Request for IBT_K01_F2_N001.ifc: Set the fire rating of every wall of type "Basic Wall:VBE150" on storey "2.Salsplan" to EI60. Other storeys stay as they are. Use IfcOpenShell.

First a look at what the model holds.

```python
import ifcopenshell
import ifcopenshell.util.element

model = ifcopenshell.open("IBT_K01_F2_N001.ifc")
print(model.schema)
storey = next(s for s in model.by_type("IfcBuildingStorey") if s.Name == "2.Salsplan")
walls = [e for e in ifcopenshell.util.element.get_decomposition(storey) if e.is_a("IfcWall")]
seen = {}
for e in walls:
    element_type = ifcopenshell.util.element.get_type(e)
    key = (element_type.Name if element_type != e and element_type else None, ifcopenshell.util.element.get_pset(e, "Pset_WallCommon", "FireRating"))
    seen[key] = seen.get(key, 0) + 1
for (name, value), count in sorted(seen.items(), key=str):
    print(count, "x", name, "|", value)
```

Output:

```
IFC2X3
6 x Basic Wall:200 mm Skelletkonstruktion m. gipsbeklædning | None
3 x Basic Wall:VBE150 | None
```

```python
import ifcopenshell
import ifcopenshell.api.pset
import ifcopenshell.util.element

model = ifcopenshell.open("IBT_K01_F2_N001.ifc")

storey = next(s for s in model.by_type("IfcBuildingStorey") if s.Name == "2.Salsplan")
walls = [e for e in ifcopenshell.util.element.get_decomposition(storey) if e.is_a("IfcWall")]

count = 0
for e in walls:
    element_type = ifcopenshell.util.element.get_type(e)
    if element_type in (None, e) or element_type.Name != "Basic Wall:VBE150":
        continue
    # add_pset returns the element's existing set when there is one.
    pset = ifcopenshell.api.pset.add_pset(model, product=e, name="Pset_WallCommon")
    ifcopenshell.api.pset.edit_pset(model, pset=pset, properties={"FireRating": "EI60"})
    count += 1

print(count, "walls updated")

model.write("IBT_K01_F2_N001_rev.ifc")
```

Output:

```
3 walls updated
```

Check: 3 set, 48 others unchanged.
